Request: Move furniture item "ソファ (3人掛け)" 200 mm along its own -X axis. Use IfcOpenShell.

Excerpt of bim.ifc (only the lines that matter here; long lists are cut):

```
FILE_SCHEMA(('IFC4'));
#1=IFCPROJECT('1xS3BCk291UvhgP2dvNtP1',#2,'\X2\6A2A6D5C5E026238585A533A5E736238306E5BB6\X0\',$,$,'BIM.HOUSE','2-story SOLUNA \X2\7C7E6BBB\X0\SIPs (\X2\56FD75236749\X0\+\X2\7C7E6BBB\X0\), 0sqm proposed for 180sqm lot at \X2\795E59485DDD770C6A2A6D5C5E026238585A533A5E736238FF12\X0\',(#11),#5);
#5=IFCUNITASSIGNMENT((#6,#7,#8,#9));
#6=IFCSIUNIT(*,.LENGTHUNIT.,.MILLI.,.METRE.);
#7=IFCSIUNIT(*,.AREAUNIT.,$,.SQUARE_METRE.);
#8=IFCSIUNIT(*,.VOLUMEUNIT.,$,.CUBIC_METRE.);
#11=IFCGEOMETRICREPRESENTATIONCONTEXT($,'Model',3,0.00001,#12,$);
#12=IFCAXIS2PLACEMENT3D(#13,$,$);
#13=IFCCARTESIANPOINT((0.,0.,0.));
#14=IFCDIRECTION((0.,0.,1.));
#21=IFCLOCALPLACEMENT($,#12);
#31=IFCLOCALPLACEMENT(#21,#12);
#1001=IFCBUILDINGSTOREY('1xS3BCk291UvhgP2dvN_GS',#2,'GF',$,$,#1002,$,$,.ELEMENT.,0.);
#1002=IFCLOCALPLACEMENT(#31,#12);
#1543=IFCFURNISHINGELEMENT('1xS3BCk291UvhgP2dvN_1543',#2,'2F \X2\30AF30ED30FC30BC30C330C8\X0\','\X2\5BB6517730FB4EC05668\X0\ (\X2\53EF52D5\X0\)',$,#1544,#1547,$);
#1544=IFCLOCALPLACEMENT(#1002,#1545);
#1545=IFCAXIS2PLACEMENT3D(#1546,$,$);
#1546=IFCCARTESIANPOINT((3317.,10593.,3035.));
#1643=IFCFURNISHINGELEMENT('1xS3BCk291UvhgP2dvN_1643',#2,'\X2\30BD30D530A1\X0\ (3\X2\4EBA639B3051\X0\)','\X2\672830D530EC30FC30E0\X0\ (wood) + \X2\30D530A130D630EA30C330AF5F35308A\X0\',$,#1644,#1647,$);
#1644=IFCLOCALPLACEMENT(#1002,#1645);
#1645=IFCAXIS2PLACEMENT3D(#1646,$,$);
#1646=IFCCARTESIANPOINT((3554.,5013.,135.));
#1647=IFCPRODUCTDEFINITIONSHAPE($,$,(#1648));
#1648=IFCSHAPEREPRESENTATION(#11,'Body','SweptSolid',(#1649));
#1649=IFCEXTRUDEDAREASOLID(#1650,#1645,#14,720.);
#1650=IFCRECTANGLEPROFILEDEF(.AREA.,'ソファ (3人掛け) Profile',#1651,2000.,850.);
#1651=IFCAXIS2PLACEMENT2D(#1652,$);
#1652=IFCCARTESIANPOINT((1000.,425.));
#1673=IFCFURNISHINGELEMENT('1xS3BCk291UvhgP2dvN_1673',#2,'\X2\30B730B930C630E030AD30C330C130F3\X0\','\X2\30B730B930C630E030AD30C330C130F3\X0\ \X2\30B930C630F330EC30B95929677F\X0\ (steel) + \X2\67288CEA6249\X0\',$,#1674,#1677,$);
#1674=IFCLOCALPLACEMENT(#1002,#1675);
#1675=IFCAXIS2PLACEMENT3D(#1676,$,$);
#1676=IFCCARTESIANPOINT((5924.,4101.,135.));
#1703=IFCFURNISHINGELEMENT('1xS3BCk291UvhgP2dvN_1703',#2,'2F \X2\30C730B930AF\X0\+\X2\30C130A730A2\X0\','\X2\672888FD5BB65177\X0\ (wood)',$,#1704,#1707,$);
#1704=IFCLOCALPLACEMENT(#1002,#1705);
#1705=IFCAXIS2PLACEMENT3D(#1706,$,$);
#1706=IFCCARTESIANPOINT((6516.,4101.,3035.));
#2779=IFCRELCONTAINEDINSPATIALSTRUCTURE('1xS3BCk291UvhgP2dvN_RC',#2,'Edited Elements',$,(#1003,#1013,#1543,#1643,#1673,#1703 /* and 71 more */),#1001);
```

```python
import ifcopenshell
import ifcopenshell.api.geometry
import ifcopenshell.util.placement

model = ifcopenshell.open("bim.ifc")

item = model.by_guid("1xS3BCk291UvhgP2dvN_1643")
matrix = ifcopenshell.util.placement.get_local_placement(item.ObjectPlacement)
matrix[:3, 3] -= matrix[:3, 0] * 200.0
ifcopenshell.api.geometry.edit_object_placement(model, product=item, matrix=matrix, is_si=False)

print(ifcopenshell.util.placement.get_local_placement(item.ObjectPlacement).round(3) + 0.0)

model.write("bim_rev.ifc")
```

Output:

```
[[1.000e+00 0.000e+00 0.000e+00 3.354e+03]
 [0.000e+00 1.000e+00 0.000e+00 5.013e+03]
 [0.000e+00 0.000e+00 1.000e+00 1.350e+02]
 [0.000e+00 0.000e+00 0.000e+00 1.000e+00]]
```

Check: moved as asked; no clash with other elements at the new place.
